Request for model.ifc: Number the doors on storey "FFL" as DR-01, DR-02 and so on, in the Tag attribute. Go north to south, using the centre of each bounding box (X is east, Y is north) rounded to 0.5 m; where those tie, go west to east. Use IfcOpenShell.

First a look at what the model holds.

```python
import ifcopenshell
import ifcopenshell.util.element
import ifcopenshell.util.placement

model = ifcopenshell.open("model.ifc")
print(model.schema)
storey = next(s for s in model.by_type("IfcBuildingStorey") if s.Name == "FFL")
doors = [e for e in ifcopenshell.util.element.get_decomposition(storey) if e.is_a("IfcDoor")]
for e in sorted(doors, key=lambda e: e.id()):
    origin = ifcopenshell.util.placement.get_local_placement(e.ObjectPlacement)[:3, 3]
    print(e.id(), e.Tag, e.Name, origin.round(2) + 0.0, sep=" | ")
```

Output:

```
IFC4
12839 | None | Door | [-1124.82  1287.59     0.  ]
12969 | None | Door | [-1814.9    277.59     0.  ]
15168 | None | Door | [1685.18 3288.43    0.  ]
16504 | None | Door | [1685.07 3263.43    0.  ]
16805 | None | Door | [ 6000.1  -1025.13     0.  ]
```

```python
import ifcopenshell
import ifcopenshell.geom
import ifcopenshell.util.element
import ifcopenshell.util.shape

model = ifcopenshell.open("model.ifc")
settings = ifcopenshell.geom.settings()
settings.set("use-world-coords", True)


def centre(element):
    shape = ifcopenshell.geom.create_shape(settings, element)
    return ifcopenshell.util.shape.get_bbox_centroid(shape.geometry)


storey = next(s for s in model.by_type("IfcBuildingStorey") if s.Name == "FFL")
doors = [e for e in ifcopenshell.util.element.get_decomposition(storey) if e.is_a("IfcDoor")]

# Insertion points can sit at a corner or the storey origin, so sort by the geometry (in metres).
centres = {e: centre(e) for e in doors}
doors.sort(key=lambda e: (-round(centres[e][1] / 0.5), centres[e][0]))

for i, e in enumerate(doors, start=1):
    number = f"DR-{i:02d}"
    e.Tag = number
    print(e.id(), number)

model.write("model_updated.ifc")
```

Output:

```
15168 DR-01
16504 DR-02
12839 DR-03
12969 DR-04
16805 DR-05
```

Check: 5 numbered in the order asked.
